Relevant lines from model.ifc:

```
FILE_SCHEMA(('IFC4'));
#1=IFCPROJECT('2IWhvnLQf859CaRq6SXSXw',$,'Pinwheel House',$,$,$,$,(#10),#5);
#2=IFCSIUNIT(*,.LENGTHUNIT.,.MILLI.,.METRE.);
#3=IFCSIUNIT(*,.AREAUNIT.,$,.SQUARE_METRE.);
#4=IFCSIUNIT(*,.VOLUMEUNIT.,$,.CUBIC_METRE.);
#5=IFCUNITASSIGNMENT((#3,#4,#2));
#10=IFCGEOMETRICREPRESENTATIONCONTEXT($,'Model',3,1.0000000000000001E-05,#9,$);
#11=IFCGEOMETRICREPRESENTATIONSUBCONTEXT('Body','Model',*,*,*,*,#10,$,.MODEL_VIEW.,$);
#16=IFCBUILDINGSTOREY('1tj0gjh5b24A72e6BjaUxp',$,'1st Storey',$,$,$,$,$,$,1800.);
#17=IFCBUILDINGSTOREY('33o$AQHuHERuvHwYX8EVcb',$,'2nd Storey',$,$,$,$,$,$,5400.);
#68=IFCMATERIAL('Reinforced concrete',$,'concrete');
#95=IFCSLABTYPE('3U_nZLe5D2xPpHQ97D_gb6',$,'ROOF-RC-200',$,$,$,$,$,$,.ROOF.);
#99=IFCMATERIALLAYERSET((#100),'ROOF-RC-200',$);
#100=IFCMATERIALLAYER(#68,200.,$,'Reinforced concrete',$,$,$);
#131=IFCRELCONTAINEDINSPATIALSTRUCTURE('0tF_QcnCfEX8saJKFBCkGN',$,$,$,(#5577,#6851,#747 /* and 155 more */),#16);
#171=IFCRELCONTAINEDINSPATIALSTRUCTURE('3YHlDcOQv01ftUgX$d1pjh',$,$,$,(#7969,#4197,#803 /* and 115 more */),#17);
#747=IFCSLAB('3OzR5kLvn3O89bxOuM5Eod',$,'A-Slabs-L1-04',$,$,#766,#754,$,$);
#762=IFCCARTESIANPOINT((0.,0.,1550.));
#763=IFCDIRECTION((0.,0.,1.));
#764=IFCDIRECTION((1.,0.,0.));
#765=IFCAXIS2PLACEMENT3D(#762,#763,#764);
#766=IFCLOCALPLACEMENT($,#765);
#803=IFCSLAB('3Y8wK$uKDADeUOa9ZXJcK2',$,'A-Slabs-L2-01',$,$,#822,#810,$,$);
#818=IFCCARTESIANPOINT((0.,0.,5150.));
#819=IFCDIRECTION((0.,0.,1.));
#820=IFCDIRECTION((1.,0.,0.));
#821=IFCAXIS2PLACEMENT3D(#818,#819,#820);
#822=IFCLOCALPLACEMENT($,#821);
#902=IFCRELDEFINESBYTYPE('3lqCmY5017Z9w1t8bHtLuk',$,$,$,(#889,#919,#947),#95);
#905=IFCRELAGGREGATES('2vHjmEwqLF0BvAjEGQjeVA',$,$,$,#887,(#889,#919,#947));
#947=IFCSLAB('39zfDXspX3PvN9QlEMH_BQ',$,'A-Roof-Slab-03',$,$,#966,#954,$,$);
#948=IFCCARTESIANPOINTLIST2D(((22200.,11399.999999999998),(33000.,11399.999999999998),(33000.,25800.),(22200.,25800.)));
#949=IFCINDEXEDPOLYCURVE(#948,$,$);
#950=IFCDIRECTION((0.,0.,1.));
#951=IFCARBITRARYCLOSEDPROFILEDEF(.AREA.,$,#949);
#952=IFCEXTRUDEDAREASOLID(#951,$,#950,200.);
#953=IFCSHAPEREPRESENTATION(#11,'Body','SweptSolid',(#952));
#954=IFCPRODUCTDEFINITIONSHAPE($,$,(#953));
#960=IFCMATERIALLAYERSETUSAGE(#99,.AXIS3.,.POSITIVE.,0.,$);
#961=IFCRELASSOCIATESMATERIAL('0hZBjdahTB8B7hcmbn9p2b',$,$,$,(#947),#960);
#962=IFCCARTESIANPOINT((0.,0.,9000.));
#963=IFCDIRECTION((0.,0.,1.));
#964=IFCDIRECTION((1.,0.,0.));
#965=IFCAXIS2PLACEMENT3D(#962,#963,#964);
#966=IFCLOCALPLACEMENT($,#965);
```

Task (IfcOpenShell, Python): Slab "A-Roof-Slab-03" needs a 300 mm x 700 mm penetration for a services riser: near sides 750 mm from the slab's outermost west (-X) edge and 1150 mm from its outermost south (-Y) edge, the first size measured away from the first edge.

```python
import numpy as np
import ifcopenshell
import ifcopenshell.api.feature
import ifcopenshell.api.geometry
import ifcopenshell.api.root
import ifcopenshell.geom
import ifcopenshell.util.placement
import ifcopenshell.util.representation
import ifcopenshell.util.shape
import ifcopenshell.util.unit

model = ifcopenshell.open("model.ifc")
unit_scale = ifcopenshell.util.unit.calculate_unit_scale(model)
settings = ifcopenshell.geom.settings()


def volume(element):
    """Net volume in cubic metres, openings subtracted."""
    shape = ifcopenshell.geom.create_shape(settings, element)
    return ifcopenshell.util.shape.get_volume(shape.geometry)


slab = model.by_guid("39zfDXspX3PvN9QlEMH_BQ")
before = volume(slab)

# Extent in the slab's own axes, in metres. The edges named are its -X and -Y sides.
slab_shape = ifcopenshell.geom.create_shape(settings, slab)
vertices = ifcopenshell.util.shape.get_vertices(slab_shape.geometry)
x_min, y_min, bottom = vertices.min(axis=0)
top = vertices[:, 2].max()

opening = ifcopenshell.api.root.create_entity(model, ifc_class="IfcOpeningElement", name="Services riser opening", predefined_type="OPENING")
context = ifcopenshell.util.representation.get_context(model, "Model", "Body", "MODEL_VIEW")
width, depth = 0.3, 0.7
outline = [(0.0, 0.0), (width, 0.0), (width, depth), (0.0, depth), (0.0, 0.0)]
# Overshoot both faces by 50 mm so the cut is clean.
shape = ifcopenshell.api.geometry.add_slab_representation(
    model, context=context, depth=top - bottom + 0.1, polyline=outline
)
ifcopenshell.api.geometry.assign_representation(model, product=opening, representation=shape)

matrix = ifcopenshell.util.placement.get_local_placement(slab.ObjectPlacement)
matrix[:, 3] = matrix @ np.append(np.array([x_min + 0.75, y_min + 1.15, bottom - 0.05]) / unit_scale, 1.0)
ifcopenshell.api.geometry.edit_object_placement(model, product=opening, matrix=matrix, is_si=False)
ifcopenshell.api.feature.add_feature(model, feature=opening, element=slab)

after = volume(slab)

print(f"slab volume {before:.3f} -> {after:.3f} m3")

model.write("model_edited.ifc")
```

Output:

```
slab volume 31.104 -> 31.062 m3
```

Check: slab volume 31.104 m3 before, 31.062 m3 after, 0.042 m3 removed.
